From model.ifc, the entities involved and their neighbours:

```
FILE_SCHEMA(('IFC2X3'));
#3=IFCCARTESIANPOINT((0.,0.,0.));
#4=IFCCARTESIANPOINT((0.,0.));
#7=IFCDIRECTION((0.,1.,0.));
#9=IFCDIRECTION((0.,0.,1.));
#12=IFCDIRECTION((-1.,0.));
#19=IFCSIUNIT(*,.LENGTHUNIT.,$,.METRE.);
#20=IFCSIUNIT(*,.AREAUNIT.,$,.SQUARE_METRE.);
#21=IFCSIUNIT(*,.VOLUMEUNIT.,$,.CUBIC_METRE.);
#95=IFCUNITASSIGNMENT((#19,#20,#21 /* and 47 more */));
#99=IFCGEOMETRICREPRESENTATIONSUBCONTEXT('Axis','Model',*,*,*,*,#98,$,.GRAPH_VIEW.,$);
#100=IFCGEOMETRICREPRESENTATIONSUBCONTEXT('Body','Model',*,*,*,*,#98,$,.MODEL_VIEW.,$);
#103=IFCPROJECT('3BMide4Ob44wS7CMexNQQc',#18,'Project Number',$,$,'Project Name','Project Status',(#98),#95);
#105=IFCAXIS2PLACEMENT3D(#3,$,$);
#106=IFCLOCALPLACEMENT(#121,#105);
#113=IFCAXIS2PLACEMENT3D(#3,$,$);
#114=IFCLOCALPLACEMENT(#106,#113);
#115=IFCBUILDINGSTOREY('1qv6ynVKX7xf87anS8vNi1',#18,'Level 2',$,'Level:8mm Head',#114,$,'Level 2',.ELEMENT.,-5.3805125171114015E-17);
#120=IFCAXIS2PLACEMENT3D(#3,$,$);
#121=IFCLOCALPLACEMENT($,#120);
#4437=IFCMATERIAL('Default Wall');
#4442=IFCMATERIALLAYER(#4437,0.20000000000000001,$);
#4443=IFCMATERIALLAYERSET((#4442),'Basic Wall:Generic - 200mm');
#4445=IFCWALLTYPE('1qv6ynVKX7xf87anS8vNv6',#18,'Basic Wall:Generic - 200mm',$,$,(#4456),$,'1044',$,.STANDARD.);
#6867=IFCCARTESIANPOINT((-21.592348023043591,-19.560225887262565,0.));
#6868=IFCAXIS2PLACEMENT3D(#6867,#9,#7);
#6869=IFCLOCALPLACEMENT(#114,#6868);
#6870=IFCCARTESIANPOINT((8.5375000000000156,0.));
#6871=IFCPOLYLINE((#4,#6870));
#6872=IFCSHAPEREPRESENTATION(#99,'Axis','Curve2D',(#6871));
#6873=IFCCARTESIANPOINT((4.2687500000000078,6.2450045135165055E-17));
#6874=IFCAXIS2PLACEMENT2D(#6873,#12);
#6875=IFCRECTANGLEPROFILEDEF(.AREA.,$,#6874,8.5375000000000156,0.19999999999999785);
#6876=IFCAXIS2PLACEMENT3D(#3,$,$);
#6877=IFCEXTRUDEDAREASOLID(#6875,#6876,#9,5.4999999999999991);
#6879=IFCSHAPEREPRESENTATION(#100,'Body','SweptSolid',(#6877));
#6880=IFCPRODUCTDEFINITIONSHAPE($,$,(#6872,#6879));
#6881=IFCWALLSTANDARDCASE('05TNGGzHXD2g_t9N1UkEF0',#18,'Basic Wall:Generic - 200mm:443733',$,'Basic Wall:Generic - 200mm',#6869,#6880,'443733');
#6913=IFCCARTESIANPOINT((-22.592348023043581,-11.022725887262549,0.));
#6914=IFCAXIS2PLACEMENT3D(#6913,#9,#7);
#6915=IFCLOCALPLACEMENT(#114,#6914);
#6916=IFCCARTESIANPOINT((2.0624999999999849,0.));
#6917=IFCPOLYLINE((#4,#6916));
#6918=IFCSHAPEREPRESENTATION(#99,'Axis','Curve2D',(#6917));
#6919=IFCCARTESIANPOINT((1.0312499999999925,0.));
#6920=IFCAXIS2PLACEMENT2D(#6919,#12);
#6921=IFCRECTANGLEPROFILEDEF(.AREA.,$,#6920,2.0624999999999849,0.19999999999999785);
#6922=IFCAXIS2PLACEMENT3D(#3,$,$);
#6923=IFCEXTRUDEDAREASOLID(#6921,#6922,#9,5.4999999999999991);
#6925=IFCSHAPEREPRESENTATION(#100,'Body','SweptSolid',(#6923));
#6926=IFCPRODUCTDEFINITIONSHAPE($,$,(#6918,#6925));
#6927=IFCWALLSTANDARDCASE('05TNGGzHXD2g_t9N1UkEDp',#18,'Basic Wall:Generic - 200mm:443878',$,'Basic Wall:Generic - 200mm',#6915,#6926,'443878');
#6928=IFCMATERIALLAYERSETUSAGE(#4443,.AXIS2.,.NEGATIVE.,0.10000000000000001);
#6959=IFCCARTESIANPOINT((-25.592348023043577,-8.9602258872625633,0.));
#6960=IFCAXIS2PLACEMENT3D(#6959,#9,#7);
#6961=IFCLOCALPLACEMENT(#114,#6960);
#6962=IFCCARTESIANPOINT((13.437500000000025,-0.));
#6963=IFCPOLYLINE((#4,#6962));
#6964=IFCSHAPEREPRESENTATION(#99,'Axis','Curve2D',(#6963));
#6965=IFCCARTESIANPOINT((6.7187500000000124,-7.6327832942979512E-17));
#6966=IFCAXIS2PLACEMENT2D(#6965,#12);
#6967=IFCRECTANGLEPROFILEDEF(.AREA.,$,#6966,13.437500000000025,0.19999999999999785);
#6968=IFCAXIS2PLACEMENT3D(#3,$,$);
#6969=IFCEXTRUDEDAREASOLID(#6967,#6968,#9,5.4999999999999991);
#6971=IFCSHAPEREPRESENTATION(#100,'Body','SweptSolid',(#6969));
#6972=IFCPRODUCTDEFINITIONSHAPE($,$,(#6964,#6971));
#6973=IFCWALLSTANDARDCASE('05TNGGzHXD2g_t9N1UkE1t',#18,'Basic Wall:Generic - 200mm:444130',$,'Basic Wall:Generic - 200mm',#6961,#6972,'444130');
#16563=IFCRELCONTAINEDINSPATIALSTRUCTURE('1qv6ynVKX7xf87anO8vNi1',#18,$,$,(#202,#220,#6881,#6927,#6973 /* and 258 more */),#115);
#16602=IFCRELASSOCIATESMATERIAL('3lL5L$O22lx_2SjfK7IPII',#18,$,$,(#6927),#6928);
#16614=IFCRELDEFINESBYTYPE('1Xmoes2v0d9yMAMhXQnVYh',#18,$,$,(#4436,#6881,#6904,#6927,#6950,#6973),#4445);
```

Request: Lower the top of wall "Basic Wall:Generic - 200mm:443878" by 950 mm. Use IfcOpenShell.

```python
import ifcopenshell
import ifcopenshell.geom
import ifcopenshell.util.representation
import ifcopenshell.util.shape
import ifcopenshell.util.unit

model = ifcopenshell.open("model.ifc")
unit_scale = ifcopenshell.util.unit.calculate_unit_scale(model)
settings = ifcopenshell.geom.settings()


def volume(element):
    """Net volume in cubic metres, openings subtracted."""
    shape = ifcopenshell.geom.create_shape(settings, element)
    return ifcopenshell.util.shape.get_volume(shape.geometry)


wall = model.by_guid("05TNGGzHXD2g_t9N1UkEDp")
before = volume(wall)

body = ifcopenshell.util.representation.get_representation(wall, "Model", "Body")
solid = body.Items[0]
old_height = solid.Depth
solid.Depth -= 0.95 / unit_scale
after = volume(wall)

print(f"height {old_height:g} -> {solid.Depth:g}, volume {before:.3f} -> {after:.3f} m3")

model.write("model_updated.ifc")
```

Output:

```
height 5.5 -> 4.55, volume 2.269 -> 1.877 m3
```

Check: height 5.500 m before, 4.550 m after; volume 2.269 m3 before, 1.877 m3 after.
